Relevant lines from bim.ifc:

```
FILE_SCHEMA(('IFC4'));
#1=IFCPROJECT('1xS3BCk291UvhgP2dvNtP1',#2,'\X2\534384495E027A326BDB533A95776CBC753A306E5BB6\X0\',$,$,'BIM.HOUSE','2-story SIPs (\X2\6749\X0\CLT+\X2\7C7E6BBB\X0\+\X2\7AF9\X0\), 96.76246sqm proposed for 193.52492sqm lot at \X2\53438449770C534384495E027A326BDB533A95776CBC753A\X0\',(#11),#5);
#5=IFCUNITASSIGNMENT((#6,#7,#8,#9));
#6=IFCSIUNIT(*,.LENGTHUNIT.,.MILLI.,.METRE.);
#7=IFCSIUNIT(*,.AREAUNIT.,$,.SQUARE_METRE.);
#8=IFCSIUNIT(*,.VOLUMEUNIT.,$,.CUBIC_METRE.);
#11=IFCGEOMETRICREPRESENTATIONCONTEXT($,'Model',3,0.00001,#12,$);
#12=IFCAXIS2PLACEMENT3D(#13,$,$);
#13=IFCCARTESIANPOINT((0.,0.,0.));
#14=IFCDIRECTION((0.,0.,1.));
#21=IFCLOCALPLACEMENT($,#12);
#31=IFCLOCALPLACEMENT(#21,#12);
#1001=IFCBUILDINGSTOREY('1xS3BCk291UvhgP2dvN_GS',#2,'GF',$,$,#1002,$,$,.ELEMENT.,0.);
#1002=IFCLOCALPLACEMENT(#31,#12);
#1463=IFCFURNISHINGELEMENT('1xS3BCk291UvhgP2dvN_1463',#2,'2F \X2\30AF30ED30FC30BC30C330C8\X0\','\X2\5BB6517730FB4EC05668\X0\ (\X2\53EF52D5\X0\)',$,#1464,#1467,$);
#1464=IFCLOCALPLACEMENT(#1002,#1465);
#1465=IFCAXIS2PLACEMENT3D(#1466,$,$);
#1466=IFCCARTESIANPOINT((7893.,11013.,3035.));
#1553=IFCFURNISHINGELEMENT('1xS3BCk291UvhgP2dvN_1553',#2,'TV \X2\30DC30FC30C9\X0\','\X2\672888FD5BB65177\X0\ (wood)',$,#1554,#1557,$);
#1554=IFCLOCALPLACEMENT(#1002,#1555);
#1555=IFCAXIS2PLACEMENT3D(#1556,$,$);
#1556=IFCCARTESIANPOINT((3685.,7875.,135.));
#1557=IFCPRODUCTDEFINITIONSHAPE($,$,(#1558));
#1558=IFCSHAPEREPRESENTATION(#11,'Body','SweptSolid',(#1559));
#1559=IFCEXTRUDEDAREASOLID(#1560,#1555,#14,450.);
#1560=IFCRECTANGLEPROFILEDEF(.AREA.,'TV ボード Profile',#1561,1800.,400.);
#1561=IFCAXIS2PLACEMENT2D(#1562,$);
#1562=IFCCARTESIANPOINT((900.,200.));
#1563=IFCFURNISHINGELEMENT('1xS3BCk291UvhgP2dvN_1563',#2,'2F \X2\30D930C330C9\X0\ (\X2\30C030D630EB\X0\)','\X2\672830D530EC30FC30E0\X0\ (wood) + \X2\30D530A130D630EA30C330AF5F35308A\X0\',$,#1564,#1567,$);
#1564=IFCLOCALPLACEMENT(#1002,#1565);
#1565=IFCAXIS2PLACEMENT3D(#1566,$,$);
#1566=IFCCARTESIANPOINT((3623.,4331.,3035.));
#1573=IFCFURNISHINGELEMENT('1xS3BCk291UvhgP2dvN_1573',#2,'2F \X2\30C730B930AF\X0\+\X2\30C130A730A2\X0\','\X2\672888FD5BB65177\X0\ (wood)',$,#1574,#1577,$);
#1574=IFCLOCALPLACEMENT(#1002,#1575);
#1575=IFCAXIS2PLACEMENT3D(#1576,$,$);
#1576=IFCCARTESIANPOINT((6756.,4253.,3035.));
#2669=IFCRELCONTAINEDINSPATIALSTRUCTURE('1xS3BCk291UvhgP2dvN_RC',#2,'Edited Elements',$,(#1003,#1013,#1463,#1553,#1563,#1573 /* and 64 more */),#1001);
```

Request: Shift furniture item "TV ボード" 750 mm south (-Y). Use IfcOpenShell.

```python
import ifcopenshell
import ifcopenshell.api.geometry
import ifcopenshell.util.placement

model = ifcopenshell.open("bim.ifc")

item = model.by_id(1553)
matrix = ifcopenshell.util.placement.get_local_placement(item.ObjectPlacement)
matrix[1, 3] -= 750.0
ifcopenshell.api.geometry.edit_object_placement(model, product=item, matrix=matrix, is_si=False)

print(ifcopenshell.util.placement.get_local_placement(item.ObjectPlacement).round(3) + 0.0)

model.write("bim_v2.ifc")
```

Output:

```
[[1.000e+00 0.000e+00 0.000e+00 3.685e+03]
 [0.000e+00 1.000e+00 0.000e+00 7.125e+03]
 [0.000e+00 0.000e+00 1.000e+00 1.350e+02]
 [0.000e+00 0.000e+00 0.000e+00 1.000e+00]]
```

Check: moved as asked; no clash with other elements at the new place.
